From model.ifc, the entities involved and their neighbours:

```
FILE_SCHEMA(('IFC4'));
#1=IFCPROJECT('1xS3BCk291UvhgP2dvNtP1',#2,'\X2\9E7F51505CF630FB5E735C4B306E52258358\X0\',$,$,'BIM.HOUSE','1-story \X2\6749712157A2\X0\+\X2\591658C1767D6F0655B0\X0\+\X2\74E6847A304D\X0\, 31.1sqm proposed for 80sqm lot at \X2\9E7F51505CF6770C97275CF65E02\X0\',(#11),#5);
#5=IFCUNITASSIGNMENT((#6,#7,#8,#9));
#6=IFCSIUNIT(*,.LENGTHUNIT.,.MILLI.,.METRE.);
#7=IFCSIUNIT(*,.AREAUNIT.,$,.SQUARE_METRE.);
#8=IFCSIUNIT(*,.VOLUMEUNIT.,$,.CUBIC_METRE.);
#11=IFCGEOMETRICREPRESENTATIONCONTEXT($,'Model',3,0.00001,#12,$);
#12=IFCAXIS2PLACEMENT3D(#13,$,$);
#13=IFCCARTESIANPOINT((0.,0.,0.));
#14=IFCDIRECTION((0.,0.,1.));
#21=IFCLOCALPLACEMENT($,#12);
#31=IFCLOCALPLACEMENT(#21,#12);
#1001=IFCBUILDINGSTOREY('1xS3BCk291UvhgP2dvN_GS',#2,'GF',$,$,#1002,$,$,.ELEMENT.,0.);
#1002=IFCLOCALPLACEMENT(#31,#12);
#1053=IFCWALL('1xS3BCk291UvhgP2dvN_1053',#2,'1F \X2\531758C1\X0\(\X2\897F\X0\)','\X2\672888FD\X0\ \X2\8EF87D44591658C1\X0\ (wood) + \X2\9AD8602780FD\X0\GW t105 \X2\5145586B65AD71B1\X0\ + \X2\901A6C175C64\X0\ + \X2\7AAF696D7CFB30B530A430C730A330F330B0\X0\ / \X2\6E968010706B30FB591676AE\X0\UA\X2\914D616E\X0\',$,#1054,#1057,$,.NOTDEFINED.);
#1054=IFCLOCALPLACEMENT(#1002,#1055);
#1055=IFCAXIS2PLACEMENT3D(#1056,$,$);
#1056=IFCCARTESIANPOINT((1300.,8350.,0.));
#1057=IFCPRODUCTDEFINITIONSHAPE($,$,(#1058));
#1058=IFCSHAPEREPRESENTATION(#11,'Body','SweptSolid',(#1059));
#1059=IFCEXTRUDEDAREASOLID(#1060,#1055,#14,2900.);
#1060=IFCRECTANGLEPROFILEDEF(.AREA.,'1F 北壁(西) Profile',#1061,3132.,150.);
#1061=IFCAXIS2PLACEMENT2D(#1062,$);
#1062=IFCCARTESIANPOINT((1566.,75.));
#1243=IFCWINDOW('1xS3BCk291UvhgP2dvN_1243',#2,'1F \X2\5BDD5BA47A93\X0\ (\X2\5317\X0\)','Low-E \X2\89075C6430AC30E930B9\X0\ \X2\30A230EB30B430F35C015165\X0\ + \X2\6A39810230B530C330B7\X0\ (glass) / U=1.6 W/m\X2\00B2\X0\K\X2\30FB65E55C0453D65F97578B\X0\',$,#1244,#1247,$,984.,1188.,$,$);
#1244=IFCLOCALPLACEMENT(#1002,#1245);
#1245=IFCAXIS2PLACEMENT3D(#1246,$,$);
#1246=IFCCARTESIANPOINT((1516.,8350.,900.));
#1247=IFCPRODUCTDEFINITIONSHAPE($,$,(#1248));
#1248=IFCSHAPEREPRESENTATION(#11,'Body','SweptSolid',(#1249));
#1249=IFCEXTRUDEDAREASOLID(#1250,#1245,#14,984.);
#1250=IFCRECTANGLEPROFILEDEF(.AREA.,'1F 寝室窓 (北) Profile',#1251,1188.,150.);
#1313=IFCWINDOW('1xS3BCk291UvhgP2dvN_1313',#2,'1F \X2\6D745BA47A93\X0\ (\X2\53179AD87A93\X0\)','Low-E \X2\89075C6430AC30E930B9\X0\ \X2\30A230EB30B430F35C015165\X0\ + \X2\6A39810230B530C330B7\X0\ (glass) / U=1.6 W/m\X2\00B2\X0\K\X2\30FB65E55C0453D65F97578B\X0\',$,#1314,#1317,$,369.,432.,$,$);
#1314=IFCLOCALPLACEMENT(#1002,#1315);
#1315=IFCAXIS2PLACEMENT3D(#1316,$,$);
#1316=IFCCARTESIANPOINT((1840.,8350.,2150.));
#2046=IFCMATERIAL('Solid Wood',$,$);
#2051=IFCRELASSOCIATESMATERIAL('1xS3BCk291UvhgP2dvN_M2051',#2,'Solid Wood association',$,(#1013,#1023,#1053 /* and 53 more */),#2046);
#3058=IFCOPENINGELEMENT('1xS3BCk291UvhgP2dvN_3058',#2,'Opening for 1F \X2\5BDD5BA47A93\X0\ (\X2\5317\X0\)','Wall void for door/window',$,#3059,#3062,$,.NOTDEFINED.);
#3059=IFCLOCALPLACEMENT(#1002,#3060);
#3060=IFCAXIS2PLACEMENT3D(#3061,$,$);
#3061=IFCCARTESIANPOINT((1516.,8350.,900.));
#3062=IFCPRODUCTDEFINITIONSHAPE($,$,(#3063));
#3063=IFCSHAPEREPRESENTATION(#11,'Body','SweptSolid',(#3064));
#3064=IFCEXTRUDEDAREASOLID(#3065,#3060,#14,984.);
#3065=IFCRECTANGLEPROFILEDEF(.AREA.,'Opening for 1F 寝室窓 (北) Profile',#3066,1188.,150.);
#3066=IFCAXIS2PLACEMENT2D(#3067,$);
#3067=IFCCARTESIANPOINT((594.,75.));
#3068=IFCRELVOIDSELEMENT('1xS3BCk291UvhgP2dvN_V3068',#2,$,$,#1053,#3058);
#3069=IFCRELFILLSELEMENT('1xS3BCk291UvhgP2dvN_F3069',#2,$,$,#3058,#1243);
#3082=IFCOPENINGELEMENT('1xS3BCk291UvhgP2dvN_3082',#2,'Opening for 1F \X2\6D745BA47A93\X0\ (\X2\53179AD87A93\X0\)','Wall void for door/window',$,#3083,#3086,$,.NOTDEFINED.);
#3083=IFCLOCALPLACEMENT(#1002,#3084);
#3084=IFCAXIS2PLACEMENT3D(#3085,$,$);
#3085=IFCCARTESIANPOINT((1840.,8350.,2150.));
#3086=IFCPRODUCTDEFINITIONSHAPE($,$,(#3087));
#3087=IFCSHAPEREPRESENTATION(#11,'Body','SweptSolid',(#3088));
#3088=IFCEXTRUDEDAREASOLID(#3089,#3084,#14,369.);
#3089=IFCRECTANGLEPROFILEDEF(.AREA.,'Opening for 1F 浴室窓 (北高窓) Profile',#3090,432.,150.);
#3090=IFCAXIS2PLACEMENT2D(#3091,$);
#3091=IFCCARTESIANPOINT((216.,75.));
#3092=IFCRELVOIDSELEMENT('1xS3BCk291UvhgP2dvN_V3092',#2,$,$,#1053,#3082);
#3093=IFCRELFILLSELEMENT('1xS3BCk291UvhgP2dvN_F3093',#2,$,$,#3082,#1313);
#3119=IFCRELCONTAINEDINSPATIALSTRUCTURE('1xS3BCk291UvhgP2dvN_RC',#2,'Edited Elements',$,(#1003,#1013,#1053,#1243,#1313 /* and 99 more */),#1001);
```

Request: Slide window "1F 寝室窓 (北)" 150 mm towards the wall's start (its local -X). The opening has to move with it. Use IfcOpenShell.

```python
import ifcopenshell
import ifcopenshell.api.geometry
import ifcopenshell.util.placement
import ifcopenshell.util.unit

model = ifcopenshell.open("model.ifc")
unit_scale = ifcopenshell.util.unit.calculate_unit_scale(model)

window = model.by_guid("1xS3BCk291UvhgP2dvN_1243")
opening = window.FillsVoids[0].RelatingOpeningElement
wall = opening.VoidsElements[0].RelatingBuildingElement

wall_matrix = ifcopenshell.util.placement.get_local_placement(wall.ObjectPlacement)
shift = wall_matrix[:3, 0] * -0.15 / unit_scale
before = ifcopenshell.util.placement.get_local_placement(window.ObjectPlacement)[:3, 3].copy()

# The window is not placed relative to its opening, so move both.
for product in (opening, window):
    matrix = ifcopenshell.util.placement.get_local_placement(product.ObjectPlacement)
    matrix[:3, 3] += shift
    ifcopenshell.api.geometry.edit_object_placement(model, product=product, matrix=matrix, is_si=False)

after = ifcopenshell.util.placement.get_local_placement(window.ObjectPlacement)[:3, 3]
print("window moved by", (after - before).round(3) + 0.0)

model.write("model_updated.ifc")
```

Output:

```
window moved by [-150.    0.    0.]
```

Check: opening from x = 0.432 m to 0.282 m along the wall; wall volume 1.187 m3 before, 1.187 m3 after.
